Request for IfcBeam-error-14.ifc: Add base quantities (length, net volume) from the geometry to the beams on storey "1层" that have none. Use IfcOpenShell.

First a look at what the model holds.

```python
import ifcopenshell
import ifcopenshell.util.element
import ifcopenshell.util.unit

model = ifcopenshell.open("IfcBeam-error-14.ifc")
print(model.schema)
for unit_type in ("LENGTHUNIT", "AREAUNIT", "VOLUMEUNIT"):
    print(unit_type, ifcopenshell.util.unit.calculate_unit_scale(model, unit_type))
storey = next(s for s in model.by_type("IfcBuildingStorey") if s.Name == "1层")
beams = [e for e in ifcopenshell.util.element.get_decomposition(storey) if e.is_a("IfcBeam")]
for e in sorted(beams, key=lambda e: e.id()):
    print(e.id(), e.is_a(), e.Name, list(ifcopenshell.util.element.get_psets(e, qtos_only=True)), sep=" | ")
```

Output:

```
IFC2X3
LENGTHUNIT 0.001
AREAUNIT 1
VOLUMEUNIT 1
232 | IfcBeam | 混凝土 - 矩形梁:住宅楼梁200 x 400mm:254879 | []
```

```python
import ifcopenshell
import ifcopenshell.api.pset
import ifcopenshell.geom
import ifcopenshell.util.element
import ifcopenshell.util.shape
import ifcopenshell.util.unit

model = ifcopenshell.open("IfcBeam-error-14.ifc")
unit_scale = ifcopenshell.util.unit.calculate_unit_scale(model)
volume_scale = ifcopenshell.util.unit.calculate_unit_scale(model, "VOLUMEUNIT")
settings = ifcopenshell.geom.settings()

storey = next(s for s in model.by_type("IfcBuildingStorey") if s.Name == "1层")
beams = [e for e in ifcopenshell.util.element.get_decomposition(storey) if e.is_a("IfcBeam")]

for e in sorted(beams, key=lambda e: e.id()):
    if ifcopenshell.util.element.get_psets(e, qtos_only=True, should_inherit=False):
        continue
    # Geometry comes back in metres, in the element's own axes.
    shape = ifcopenshell.geom.create_shape(settings, e)
    values = {
        "Length": ifcopenshell.util.shape.get_max_xyz(shape.geometry) / unit_scale,
        "NetVolume": ifcopenshell.util.shape.get_volume(shape.geometry) / volume_scale,
    }
    qto = ifcopenshell.api.pset.add_qto(model, product=e, name="BaseQuantities")
    ifcopenshell.api.pset.edit_qto(model, qto=qto, properties=values)
    print(e.id(), {k: round(v, 3) for k, v in values.items()})

model.write("IfcBeam-error-14_edited.ifc")
```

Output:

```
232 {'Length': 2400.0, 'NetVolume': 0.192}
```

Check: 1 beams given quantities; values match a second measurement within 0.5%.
